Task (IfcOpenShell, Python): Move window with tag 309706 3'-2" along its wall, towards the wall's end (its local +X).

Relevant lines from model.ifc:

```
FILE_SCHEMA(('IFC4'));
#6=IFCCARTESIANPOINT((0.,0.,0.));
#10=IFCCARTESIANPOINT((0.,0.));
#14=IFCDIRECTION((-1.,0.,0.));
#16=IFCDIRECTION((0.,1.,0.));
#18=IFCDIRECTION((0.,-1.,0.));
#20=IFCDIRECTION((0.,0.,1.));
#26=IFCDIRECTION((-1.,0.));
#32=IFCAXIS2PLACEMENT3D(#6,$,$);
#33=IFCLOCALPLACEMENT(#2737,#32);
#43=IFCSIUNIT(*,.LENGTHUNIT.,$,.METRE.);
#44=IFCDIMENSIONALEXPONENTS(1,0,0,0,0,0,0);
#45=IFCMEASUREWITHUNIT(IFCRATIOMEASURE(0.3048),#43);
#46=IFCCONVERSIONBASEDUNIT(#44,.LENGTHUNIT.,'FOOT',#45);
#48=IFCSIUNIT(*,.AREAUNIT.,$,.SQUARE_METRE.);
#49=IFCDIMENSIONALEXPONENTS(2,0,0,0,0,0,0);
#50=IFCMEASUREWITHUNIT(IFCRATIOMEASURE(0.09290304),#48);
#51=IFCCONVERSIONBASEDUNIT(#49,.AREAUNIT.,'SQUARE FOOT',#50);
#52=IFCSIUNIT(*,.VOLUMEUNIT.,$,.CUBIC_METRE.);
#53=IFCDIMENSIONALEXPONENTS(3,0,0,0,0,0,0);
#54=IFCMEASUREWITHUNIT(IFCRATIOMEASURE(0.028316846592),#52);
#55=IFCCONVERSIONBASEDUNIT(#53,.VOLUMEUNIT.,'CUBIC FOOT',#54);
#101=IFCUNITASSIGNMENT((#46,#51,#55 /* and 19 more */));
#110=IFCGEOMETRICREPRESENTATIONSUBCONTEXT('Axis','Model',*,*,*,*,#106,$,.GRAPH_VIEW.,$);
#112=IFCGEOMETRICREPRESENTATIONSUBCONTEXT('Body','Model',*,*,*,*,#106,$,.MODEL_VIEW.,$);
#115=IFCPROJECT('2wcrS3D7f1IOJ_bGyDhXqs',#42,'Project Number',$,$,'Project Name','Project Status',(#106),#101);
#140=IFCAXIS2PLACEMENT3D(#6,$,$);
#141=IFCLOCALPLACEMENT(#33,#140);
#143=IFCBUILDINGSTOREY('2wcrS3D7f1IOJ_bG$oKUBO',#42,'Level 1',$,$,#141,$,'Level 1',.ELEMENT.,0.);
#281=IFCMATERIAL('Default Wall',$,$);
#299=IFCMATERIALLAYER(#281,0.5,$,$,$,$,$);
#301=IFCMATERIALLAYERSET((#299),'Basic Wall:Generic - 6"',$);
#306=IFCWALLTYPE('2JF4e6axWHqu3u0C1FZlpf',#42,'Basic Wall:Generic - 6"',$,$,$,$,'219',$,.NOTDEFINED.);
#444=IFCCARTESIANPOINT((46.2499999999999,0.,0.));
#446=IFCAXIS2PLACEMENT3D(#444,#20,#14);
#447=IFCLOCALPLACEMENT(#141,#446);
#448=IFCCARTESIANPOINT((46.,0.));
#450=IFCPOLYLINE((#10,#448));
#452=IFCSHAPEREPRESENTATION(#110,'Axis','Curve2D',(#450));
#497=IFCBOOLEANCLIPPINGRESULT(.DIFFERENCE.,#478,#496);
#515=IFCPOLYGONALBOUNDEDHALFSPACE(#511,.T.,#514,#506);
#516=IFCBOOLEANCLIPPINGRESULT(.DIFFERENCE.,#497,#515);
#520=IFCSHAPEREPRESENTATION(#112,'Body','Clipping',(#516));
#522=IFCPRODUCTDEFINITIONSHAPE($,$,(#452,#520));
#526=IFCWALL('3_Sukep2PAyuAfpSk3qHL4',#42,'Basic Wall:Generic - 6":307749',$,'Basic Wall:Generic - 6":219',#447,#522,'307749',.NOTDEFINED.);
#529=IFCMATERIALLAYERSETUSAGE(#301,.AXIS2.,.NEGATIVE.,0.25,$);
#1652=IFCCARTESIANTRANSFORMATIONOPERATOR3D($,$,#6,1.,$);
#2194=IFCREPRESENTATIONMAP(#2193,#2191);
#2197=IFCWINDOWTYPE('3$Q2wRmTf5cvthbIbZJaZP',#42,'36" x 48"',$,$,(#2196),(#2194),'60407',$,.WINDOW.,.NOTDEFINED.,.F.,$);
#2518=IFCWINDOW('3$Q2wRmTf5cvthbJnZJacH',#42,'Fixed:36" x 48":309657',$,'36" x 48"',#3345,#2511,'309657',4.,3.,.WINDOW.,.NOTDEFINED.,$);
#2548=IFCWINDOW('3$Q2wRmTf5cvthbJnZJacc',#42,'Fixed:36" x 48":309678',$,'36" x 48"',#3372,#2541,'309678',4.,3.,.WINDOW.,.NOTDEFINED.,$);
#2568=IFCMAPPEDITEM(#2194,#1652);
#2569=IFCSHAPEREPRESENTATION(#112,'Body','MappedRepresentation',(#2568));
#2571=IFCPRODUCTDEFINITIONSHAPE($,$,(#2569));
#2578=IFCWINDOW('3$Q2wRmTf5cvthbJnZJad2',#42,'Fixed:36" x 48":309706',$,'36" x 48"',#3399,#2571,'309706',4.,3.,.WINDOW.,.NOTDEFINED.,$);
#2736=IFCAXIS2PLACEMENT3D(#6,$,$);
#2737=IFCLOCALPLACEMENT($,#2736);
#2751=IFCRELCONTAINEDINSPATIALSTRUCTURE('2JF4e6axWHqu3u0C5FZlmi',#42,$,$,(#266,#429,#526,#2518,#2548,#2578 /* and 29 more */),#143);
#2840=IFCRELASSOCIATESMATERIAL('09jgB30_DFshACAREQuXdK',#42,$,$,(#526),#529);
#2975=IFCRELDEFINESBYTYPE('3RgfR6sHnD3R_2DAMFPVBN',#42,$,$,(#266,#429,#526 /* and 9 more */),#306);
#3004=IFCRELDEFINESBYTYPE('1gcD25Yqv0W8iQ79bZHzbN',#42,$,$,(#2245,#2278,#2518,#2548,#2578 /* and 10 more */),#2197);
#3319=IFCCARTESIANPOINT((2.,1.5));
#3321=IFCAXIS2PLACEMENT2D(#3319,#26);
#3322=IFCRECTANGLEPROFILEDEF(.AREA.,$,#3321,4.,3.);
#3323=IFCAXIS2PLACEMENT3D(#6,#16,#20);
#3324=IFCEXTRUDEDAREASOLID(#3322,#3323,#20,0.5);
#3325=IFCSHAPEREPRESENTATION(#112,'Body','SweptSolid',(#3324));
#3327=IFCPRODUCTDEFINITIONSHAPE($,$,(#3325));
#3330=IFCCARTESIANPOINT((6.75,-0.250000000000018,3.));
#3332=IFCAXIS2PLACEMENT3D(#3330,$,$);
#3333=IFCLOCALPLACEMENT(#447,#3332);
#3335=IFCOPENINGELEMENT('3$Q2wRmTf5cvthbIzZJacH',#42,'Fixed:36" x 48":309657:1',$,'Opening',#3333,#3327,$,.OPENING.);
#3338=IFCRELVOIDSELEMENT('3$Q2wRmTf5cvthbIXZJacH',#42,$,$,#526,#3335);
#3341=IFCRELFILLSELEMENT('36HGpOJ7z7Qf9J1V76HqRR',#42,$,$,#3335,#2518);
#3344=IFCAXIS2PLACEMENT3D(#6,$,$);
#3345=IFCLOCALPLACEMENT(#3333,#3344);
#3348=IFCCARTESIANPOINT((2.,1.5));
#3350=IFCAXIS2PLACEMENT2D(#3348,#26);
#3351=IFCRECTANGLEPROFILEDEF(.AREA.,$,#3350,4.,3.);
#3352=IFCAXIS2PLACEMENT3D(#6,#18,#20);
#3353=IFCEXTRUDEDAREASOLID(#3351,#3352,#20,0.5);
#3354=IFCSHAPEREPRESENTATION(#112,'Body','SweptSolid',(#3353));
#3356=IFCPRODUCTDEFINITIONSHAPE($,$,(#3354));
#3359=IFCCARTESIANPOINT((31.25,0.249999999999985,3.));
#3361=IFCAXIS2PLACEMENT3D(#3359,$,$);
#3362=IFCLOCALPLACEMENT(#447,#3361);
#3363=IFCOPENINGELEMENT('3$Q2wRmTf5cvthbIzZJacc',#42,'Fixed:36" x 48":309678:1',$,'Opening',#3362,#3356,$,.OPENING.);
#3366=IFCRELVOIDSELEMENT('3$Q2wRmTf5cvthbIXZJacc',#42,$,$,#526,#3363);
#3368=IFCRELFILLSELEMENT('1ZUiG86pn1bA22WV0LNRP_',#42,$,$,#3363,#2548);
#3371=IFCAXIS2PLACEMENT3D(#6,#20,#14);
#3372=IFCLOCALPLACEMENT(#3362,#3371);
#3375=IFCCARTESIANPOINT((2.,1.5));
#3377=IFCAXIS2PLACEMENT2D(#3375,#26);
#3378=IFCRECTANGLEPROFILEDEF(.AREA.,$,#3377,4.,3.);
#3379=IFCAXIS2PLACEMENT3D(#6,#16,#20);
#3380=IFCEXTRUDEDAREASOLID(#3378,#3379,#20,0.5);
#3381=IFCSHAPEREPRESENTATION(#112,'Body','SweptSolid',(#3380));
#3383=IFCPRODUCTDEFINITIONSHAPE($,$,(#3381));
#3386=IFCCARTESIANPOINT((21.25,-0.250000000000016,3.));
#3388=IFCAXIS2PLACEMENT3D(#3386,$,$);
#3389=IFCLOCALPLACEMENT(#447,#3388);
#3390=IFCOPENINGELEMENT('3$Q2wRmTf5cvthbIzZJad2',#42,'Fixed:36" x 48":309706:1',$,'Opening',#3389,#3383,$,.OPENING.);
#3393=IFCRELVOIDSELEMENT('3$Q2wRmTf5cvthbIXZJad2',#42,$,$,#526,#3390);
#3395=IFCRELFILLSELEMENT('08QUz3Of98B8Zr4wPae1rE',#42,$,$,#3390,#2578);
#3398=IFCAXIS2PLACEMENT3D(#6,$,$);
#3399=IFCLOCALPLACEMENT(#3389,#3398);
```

```python
import ifcopenshell
import ifcopenshell.api.geometry
import ifcopenshell.util.placement
import ifcopenshell.util.unit

model = ifcopenshell.open("model.ifc")
unit_scale = ifcopenshell.util.unit.calculate_unit_scale(model)

window = model.by_id(2578)
opening = window.FillsVoids[0].RelatingOpeningElement
wall = opening.VoidsElements[0].RelatingBuildingElement

wall_matrix = ifcopenshell.util.placement.get_local_placement(wall.ObjectPlacement)
shift = wall_matrix[:3, 0] * 38 * 0.0254 / unit_scale
before = ifcopenshell.util.placement.get_local_placement(window.ObjectPlacement)[:3, 3].copy()

# The window is placed relative to its opening, so it follows when the opening moves.
matrix = ifcopenshell.util.placement.get_local_placement(opening.ObjectPlacement)
matrix[:3, 3] += shift
ifcopenshell.api.geometry.edit_object_placement(
    model, product=opening, matrix=matrix, is_si=False, should_transform_children=True
)

after = ifcopenshell.util.placement.get_local_placement(window.ObjectPlacement)[:3, 3]
print("window moved by", (after - before).round(3) + 0.0)

model.write("model-out.ifc")
```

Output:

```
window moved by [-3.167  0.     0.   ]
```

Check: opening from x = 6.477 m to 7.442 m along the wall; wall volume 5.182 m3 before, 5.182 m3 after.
